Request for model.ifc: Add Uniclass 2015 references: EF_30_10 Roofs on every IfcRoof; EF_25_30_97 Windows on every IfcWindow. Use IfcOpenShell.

First a look at what the model holds.

```python
import ifcopenshell

model = ifcopenshell.open("model.ifc")
print(model.schema)
print("classifications:", [c.Name for c in model.by_type("IfcClassification")])
for ifc_class in ("IfcDoor", "IfcRoof", "IfcStair", "IfcWall", "IfcWindow"):
    print(ifc_class, len(model.by_type(ifc_class)))
```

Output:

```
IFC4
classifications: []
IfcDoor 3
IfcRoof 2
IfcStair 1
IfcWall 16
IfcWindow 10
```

```python
import ifcopenshell
import ifcopenshell.api.classification

model = ifcopenshell.open("model.ifc")

system = ifcopenshell.api.classification.add_classification(model, classification="Uniclass 2015")

codes = {
    "IfcRoof": ("EF_30_10", "Roofs"),
    "IfcWindow": ("EF_25_30_97", "Windows"),
}
for ifc_class, (code, name) in codes.items():
    products = model.by_type(ifc_class)
    ifcopenshell.api.classification.add_reference(
        model, products=products, classification=system, identification=code, name=name
    )
    print(code, len(products))

model.write("model-out.ifc")
```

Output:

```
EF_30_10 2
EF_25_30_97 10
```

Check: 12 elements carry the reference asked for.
